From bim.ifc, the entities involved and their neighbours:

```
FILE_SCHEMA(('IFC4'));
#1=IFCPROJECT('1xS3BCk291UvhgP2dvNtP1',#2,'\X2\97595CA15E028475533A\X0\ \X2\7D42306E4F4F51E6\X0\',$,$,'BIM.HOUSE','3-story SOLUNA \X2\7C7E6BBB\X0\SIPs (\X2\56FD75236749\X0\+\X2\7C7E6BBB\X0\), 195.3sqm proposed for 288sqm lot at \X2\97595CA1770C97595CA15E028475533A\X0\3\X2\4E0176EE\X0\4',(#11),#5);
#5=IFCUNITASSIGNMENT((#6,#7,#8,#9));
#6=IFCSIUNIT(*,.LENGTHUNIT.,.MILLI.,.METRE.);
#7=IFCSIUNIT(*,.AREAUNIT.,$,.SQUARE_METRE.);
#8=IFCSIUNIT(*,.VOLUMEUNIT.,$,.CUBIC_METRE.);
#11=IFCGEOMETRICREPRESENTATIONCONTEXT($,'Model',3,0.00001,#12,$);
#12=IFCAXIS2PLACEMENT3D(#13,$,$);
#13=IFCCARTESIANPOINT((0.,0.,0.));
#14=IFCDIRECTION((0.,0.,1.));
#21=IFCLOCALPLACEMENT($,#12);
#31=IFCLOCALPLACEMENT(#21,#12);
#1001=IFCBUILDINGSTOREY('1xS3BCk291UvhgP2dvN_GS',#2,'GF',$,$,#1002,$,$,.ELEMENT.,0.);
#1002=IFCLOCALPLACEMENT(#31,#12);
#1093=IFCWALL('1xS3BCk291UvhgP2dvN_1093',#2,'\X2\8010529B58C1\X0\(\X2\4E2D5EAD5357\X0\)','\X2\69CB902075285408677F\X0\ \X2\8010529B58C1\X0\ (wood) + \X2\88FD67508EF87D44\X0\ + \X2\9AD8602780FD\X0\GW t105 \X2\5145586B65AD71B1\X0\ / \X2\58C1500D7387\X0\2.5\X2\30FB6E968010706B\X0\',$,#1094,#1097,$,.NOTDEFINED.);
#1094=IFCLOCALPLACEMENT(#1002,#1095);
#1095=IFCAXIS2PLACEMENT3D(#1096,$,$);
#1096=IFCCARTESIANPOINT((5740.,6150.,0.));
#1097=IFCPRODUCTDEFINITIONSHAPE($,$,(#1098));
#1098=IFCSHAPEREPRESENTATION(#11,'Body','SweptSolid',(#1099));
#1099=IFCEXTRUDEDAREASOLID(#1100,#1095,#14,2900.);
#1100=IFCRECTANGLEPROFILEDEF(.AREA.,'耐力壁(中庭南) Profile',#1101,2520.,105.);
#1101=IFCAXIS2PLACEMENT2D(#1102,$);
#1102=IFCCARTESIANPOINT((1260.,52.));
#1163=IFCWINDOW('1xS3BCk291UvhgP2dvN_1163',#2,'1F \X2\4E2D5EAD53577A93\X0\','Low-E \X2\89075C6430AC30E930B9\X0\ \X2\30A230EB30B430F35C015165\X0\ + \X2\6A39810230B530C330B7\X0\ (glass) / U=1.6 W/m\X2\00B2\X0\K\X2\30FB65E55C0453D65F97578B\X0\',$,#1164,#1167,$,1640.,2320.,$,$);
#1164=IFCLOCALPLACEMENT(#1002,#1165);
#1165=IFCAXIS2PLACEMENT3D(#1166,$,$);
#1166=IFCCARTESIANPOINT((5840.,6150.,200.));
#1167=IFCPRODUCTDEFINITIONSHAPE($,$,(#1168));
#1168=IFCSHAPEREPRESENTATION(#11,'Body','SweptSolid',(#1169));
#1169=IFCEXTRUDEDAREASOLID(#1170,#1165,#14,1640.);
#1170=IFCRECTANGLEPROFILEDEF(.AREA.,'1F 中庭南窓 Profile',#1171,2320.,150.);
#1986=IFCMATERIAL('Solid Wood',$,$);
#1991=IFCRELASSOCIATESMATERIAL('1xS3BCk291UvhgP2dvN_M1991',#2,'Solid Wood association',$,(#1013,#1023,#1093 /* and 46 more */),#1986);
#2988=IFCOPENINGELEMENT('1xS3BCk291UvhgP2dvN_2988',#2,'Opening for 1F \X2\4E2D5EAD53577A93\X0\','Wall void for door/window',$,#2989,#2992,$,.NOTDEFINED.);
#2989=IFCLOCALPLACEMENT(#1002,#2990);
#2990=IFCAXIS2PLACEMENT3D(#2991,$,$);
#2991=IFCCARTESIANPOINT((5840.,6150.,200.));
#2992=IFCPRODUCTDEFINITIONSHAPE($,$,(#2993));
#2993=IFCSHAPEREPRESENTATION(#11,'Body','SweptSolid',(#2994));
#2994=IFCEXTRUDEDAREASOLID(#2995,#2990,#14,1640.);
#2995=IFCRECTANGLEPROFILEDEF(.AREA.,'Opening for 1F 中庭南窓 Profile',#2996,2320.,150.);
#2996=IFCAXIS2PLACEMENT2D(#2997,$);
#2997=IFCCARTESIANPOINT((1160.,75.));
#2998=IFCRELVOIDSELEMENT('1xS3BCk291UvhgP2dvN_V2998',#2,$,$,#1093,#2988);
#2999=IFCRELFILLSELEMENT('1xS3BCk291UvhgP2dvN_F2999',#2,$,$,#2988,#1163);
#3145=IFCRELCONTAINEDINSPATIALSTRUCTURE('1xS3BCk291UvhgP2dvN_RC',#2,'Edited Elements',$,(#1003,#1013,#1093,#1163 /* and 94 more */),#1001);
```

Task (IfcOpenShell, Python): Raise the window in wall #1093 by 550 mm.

```python
import numpy as np
import ifcopenshell
import ifcopenshell.api.geometry
import ifcopenshell.util.placement
import ifcopenshell.util.unit

model = ifcopenshell.open("bim.ifc")
unit_scale = ifcopenshell.util.unit.calculate_unit_scale(model)

window = model.by_guid("1xS3BCk291UvhgP2dvN_1163")
opening = window.FillsVoids[0].RelatingOpeningElement
dz = 0.55 / unit_scale

shift = np.array([0.0, 0.0, dz])
# The window is not placed relative to its opening, so move both.
for product in (opening, window):
    matrix = ifcopenshell.util.placement.get_local_placement(product.ObjectPlacement)
    matrix[:3, 3] += shift
    ifcopenshell.api.geometry.edit_object_placement(model, product=product, matrix=matrix, is_si=False)

print(f"moved by {dz * unit_scale:+.3f} m")

model.write("bim_rev.ifc")
```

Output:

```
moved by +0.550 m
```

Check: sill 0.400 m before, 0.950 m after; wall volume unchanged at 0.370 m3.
